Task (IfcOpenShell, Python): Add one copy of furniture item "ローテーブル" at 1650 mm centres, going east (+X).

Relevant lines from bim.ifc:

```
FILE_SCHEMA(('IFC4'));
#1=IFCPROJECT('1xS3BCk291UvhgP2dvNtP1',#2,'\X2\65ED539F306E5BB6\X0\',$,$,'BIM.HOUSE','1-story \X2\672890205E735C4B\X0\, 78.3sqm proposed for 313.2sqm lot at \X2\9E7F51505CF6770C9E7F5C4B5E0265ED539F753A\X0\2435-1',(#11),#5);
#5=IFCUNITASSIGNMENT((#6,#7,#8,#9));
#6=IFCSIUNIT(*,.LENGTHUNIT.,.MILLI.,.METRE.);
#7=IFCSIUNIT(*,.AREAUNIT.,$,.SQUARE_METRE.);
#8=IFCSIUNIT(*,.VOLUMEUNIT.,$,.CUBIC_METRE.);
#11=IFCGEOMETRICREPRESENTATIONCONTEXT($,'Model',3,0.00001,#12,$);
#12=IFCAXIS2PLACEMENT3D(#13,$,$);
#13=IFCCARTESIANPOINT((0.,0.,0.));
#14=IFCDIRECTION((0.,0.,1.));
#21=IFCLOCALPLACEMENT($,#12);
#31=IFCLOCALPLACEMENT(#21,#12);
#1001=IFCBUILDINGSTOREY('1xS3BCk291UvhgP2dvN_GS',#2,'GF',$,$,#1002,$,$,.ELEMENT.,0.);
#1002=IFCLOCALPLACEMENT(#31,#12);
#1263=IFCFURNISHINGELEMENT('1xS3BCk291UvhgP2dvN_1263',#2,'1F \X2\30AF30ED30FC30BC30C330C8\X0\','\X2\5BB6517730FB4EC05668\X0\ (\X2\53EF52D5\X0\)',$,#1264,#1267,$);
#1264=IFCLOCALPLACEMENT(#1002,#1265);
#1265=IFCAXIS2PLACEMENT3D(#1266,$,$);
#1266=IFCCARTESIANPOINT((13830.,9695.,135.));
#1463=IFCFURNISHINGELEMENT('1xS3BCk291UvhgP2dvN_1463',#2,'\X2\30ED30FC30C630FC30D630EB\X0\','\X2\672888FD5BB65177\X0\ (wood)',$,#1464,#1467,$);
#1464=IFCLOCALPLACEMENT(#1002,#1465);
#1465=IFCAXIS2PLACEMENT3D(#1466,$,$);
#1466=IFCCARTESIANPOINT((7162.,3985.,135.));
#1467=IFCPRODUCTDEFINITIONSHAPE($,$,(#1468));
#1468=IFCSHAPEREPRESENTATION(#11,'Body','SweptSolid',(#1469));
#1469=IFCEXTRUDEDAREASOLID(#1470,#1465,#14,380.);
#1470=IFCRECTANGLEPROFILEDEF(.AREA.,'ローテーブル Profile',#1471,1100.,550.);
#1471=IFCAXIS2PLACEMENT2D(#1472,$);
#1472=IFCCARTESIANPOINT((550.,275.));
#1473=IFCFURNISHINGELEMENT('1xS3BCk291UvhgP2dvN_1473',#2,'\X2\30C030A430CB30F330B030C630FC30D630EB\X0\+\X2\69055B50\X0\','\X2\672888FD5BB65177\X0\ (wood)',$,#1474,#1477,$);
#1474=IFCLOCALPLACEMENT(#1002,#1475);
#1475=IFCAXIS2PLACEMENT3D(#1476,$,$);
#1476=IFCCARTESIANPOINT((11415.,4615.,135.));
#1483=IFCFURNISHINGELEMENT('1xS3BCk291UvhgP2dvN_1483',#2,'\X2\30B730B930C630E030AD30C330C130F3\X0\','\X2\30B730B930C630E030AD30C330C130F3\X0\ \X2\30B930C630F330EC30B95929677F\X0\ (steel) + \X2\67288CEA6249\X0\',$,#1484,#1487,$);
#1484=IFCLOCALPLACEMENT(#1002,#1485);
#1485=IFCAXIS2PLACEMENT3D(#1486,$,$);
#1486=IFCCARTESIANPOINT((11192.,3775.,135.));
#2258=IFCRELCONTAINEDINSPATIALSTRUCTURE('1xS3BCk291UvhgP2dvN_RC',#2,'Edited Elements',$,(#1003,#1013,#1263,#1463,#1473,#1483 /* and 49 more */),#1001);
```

```python
import numpy as np
import ifcopenshell
import ifcopenshell.api.geometry
import ifcopenshell.api.root
import ifcopenshell.util.element
import ifcopenshell.util.placement
import ifcopenshell.util.unit

model = ifcopenshell.open("bim.ifc")
unit_scale = ifcopenshell.util.unit.calculate_unit_scale(model)


def reuse_history(source, copy):
    """copy_class also copies each property set's owner history, people and application; keep the originals."""
    for rel in copy.IsDefinedBy:
        if rel.is_a("IfcRelDefinesByProperties") and (history := rel.RelatingPropertyDefinition.OwnerHistory):
            rel.RelatingPropertyDefinition.OwnerHistory = source.OwnerHistory
            ifcopenshell.util.element.remove_deep2(model, history)


source = model.by_id(1463)
base = ifcopenshell.util.placement.get_local_placement(source.ObjectPlacement)
step = np.array([1.0, 0.0, 0.0]) * 1.65 / unit_scale

for i in range(1, 2):
    copy = ifcopenshell.api.root.copy_class(model, product=source)
    copy.Representation = ifcopenshell.util.element.copy_deep(
        model, source.Representation, exclude=["IfcGeometricRepresentationContext", "IfcRepresentationMap"]
    )
    reuse_history(source, copy)
    matrix = base.copy()
    matrix[:3, 3] += i * step
    print("added at", matrix[:3, 3].round(3) + 0.0)
    ifcopenshell.api.geometry.edit_object_placement(model, product=copy, matrix=matrix, is_si=False)

model.write("bim_edited.ifc")
```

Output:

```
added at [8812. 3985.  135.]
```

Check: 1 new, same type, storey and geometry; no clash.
